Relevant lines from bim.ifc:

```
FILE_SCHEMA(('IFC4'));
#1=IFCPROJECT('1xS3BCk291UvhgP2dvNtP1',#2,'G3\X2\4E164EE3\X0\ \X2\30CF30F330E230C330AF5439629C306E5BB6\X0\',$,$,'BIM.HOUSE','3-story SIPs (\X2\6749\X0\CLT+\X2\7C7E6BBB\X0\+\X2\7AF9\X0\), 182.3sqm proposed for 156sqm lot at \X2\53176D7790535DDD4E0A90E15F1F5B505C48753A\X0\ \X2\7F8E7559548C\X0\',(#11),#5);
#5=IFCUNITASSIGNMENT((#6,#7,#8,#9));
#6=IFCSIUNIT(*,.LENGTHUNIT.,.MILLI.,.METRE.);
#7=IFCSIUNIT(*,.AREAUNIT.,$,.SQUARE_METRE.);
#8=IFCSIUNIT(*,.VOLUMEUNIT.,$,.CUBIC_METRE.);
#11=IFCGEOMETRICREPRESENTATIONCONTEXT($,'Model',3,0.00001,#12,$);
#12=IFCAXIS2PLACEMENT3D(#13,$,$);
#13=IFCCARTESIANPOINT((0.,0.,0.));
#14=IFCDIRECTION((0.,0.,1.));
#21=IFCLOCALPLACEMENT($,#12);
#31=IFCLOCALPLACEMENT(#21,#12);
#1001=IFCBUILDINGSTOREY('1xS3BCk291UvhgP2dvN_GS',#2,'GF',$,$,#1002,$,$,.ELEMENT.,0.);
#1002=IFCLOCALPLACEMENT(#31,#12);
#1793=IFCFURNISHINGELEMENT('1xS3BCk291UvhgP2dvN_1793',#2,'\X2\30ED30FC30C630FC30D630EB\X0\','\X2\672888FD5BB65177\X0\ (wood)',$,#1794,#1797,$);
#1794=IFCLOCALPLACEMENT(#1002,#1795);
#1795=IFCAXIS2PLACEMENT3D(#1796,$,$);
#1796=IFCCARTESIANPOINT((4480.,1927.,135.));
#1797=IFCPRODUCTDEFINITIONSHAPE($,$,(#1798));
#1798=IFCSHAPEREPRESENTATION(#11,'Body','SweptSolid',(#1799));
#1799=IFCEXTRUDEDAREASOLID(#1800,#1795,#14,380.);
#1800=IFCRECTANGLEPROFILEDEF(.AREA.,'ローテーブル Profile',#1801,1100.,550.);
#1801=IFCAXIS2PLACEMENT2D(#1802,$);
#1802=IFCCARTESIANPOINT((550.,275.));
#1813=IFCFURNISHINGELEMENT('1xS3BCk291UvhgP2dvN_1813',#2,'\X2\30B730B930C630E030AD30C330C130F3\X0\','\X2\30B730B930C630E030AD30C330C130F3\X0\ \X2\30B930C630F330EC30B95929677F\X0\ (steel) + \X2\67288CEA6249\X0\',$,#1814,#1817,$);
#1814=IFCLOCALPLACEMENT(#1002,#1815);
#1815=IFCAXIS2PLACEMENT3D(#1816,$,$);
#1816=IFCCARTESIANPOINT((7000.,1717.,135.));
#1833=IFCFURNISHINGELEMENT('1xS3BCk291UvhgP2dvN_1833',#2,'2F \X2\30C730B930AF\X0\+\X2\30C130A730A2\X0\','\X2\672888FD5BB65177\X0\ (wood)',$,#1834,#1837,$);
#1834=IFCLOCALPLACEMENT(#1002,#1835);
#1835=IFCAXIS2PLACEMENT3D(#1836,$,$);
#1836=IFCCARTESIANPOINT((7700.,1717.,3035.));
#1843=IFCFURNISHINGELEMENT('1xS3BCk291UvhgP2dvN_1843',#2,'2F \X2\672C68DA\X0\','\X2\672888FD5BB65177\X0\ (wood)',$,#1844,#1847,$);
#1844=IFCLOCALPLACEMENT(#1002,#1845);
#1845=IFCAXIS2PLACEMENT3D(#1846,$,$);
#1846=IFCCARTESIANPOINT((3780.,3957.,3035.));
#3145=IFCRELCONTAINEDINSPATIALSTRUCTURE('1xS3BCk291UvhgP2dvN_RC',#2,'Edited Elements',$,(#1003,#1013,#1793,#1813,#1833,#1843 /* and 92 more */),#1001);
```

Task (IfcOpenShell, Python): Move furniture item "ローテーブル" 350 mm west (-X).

```python
import ifcopenshell
import ifcopenshell.api.geometry
import ifcopenshell.util.placement
import ifcopenshell.util.unit

model = ifcopenshell.open("bim.ifc")
unit_scale = ifcopenshell.util.unit.calculate_unit_scale(model)

item = model.by_id(1793)
matrix = ifcopenshell.util.placement.get_local_placement(item.ObjectPlacement)
matrix[0, 3] -= 0.35 / unit_scale
ifcopenshell.api.geometry.edit_object_placement(model, product=item, matrix=matrix, is_si=False)

print(ifcopenshell.util.placement.get_local_placement(item.ObjectPlacement).round(3) + 0.0)

model.write("bim_rev.ifc")
```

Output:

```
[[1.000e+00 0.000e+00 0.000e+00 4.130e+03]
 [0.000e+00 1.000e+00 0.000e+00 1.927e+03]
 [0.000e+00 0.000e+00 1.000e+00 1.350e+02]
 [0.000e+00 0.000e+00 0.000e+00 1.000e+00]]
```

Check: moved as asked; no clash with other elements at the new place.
